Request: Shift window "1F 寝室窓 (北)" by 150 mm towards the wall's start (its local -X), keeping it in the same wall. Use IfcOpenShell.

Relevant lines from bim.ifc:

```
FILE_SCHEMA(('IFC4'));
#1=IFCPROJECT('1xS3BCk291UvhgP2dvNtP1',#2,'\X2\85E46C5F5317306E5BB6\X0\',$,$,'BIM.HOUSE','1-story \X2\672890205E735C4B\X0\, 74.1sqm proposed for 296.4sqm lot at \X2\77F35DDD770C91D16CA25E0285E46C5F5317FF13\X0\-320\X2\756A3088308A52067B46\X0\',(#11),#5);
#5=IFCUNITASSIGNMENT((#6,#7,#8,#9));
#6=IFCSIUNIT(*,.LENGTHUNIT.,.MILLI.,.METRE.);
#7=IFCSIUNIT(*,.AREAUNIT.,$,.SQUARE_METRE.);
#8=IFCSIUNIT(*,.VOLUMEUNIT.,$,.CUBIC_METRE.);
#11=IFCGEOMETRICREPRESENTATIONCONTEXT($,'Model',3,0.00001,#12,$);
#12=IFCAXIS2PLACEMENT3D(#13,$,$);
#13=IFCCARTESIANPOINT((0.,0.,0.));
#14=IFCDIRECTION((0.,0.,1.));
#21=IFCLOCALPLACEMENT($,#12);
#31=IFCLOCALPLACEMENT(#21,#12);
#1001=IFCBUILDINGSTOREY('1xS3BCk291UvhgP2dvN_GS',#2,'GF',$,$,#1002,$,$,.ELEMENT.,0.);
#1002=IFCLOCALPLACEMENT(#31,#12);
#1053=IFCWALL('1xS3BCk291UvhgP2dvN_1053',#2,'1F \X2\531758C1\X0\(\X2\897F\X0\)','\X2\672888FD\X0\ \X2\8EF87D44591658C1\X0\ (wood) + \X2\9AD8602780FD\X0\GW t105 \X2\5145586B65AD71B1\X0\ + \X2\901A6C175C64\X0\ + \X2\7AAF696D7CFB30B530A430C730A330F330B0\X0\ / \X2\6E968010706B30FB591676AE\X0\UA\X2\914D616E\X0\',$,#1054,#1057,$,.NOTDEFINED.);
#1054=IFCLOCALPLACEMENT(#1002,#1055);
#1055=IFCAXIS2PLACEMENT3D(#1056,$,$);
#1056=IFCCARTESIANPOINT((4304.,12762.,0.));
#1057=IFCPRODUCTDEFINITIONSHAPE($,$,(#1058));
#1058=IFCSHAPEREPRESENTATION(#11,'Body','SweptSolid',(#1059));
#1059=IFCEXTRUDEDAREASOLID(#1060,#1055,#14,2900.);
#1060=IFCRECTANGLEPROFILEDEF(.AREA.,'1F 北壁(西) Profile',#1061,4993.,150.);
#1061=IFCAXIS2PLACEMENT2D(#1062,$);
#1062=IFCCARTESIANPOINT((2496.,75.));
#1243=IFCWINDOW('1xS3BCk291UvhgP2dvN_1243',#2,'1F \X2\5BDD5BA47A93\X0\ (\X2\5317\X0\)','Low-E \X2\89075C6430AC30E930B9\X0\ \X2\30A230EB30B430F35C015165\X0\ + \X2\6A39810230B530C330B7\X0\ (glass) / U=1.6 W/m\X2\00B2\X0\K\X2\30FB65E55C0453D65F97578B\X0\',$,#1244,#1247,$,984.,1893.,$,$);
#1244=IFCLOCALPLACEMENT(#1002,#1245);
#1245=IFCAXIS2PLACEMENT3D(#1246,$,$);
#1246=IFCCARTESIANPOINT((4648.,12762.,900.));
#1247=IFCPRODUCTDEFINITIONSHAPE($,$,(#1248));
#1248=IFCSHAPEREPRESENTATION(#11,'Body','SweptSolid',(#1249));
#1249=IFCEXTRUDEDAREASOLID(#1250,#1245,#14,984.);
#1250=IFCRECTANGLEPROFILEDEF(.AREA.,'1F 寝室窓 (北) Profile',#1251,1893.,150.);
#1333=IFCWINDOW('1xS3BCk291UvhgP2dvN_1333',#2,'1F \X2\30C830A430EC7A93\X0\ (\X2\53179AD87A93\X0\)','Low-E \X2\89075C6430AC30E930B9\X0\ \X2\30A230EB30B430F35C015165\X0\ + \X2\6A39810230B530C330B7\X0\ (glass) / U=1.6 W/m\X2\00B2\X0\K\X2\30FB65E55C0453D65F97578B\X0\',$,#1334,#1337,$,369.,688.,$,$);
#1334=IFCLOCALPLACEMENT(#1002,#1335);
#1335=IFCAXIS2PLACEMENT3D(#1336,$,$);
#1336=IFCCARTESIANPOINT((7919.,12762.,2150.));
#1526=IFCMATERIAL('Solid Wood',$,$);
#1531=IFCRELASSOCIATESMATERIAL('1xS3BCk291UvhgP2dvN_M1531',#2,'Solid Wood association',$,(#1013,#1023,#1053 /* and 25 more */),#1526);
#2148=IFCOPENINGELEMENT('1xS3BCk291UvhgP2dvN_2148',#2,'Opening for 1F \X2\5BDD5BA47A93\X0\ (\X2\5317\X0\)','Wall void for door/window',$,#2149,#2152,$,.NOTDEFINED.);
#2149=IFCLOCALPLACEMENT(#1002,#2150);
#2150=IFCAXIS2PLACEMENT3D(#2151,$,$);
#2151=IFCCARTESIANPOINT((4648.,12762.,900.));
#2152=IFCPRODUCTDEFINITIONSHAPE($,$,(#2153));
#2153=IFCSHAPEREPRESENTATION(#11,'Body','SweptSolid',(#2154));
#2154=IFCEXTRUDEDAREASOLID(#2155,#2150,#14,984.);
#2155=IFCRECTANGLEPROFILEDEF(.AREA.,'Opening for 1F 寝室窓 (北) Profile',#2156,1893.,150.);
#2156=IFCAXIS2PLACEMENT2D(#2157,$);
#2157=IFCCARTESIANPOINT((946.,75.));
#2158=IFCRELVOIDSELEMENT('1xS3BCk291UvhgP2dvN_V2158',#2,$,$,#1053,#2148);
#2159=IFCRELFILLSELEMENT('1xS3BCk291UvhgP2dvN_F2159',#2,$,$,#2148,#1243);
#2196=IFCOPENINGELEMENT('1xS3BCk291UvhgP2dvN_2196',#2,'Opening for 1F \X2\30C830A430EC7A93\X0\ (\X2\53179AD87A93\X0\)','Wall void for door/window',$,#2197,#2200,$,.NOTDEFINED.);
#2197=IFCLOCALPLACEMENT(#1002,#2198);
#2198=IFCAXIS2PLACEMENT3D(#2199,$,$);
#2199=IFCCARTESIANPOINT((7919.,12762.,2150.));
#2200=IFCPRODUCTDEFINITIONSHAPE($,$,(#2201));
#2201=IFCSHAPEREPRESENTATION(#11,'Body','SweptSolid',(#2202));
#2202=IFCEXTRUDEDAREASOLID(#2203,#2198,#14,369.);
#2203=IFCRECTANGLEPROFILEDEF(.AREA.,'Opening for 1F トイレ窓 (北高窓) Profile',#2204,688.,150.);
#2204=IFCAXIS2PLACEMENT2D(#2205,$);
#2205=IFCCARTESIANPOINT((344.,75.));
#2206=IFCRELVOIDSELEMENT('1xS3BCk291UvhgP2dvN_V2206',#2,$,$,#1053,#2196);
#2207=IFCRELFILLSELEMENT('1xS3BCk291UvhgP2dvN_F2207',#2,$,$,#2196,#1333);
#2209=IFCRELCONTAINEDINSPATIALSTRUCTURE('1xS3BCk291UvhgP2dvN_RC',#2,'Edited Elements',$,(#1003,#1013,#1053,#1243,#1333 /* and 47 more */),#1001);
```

```python
import ifcopenshell
import ifcopenshell.api.geometry
import ifcopenshell.util.placement
import ifcopenshell.util.unit

model = ifcopenshell.open("bim.ifc")
unit_scale = ifcopenshell.util.unit.calculate_unit_scale(model)

window = model.by_guid("1xS3BCk291UvhgP2dvN_1243")
opening = window.FillsVoids[0].RelatingOpeningElement
wall = opening.VoidsElements[0].RelatingBuildingElement

wall_matrix = ifcopenshell.util.placement.get_local_placement(wall.ObjectPlacement)
shift = wall_matrix[:3, 0] * -0.15 / unit_scale
before = ifcopenshell.util.placement.get_local_placement(window.ObjectPlacement)[:3, 3].copy()

# The window is not placed relative to its opening, so move both.
for product in (opening, window):
    matrix = ifcopenshell.util.placement.get_local_placement(product.ObjectPlacement)
    matrix[:3, 3] += shift
    ifcopenshell.api.geometry.edit_object_placement(model, product=product, matrix=matrix, is_si=False)

after = ifcopenshell.util.placement.get_local_placement(window.ObjectPlacement)[:3, 3]
print("window moved by", (after - before).round(3) + 0.0)

model.write("bim_v2.ifc")
```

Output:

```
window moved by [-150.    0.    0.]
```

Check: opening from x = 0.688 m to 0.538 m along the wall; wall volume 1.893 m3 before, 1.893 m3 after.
